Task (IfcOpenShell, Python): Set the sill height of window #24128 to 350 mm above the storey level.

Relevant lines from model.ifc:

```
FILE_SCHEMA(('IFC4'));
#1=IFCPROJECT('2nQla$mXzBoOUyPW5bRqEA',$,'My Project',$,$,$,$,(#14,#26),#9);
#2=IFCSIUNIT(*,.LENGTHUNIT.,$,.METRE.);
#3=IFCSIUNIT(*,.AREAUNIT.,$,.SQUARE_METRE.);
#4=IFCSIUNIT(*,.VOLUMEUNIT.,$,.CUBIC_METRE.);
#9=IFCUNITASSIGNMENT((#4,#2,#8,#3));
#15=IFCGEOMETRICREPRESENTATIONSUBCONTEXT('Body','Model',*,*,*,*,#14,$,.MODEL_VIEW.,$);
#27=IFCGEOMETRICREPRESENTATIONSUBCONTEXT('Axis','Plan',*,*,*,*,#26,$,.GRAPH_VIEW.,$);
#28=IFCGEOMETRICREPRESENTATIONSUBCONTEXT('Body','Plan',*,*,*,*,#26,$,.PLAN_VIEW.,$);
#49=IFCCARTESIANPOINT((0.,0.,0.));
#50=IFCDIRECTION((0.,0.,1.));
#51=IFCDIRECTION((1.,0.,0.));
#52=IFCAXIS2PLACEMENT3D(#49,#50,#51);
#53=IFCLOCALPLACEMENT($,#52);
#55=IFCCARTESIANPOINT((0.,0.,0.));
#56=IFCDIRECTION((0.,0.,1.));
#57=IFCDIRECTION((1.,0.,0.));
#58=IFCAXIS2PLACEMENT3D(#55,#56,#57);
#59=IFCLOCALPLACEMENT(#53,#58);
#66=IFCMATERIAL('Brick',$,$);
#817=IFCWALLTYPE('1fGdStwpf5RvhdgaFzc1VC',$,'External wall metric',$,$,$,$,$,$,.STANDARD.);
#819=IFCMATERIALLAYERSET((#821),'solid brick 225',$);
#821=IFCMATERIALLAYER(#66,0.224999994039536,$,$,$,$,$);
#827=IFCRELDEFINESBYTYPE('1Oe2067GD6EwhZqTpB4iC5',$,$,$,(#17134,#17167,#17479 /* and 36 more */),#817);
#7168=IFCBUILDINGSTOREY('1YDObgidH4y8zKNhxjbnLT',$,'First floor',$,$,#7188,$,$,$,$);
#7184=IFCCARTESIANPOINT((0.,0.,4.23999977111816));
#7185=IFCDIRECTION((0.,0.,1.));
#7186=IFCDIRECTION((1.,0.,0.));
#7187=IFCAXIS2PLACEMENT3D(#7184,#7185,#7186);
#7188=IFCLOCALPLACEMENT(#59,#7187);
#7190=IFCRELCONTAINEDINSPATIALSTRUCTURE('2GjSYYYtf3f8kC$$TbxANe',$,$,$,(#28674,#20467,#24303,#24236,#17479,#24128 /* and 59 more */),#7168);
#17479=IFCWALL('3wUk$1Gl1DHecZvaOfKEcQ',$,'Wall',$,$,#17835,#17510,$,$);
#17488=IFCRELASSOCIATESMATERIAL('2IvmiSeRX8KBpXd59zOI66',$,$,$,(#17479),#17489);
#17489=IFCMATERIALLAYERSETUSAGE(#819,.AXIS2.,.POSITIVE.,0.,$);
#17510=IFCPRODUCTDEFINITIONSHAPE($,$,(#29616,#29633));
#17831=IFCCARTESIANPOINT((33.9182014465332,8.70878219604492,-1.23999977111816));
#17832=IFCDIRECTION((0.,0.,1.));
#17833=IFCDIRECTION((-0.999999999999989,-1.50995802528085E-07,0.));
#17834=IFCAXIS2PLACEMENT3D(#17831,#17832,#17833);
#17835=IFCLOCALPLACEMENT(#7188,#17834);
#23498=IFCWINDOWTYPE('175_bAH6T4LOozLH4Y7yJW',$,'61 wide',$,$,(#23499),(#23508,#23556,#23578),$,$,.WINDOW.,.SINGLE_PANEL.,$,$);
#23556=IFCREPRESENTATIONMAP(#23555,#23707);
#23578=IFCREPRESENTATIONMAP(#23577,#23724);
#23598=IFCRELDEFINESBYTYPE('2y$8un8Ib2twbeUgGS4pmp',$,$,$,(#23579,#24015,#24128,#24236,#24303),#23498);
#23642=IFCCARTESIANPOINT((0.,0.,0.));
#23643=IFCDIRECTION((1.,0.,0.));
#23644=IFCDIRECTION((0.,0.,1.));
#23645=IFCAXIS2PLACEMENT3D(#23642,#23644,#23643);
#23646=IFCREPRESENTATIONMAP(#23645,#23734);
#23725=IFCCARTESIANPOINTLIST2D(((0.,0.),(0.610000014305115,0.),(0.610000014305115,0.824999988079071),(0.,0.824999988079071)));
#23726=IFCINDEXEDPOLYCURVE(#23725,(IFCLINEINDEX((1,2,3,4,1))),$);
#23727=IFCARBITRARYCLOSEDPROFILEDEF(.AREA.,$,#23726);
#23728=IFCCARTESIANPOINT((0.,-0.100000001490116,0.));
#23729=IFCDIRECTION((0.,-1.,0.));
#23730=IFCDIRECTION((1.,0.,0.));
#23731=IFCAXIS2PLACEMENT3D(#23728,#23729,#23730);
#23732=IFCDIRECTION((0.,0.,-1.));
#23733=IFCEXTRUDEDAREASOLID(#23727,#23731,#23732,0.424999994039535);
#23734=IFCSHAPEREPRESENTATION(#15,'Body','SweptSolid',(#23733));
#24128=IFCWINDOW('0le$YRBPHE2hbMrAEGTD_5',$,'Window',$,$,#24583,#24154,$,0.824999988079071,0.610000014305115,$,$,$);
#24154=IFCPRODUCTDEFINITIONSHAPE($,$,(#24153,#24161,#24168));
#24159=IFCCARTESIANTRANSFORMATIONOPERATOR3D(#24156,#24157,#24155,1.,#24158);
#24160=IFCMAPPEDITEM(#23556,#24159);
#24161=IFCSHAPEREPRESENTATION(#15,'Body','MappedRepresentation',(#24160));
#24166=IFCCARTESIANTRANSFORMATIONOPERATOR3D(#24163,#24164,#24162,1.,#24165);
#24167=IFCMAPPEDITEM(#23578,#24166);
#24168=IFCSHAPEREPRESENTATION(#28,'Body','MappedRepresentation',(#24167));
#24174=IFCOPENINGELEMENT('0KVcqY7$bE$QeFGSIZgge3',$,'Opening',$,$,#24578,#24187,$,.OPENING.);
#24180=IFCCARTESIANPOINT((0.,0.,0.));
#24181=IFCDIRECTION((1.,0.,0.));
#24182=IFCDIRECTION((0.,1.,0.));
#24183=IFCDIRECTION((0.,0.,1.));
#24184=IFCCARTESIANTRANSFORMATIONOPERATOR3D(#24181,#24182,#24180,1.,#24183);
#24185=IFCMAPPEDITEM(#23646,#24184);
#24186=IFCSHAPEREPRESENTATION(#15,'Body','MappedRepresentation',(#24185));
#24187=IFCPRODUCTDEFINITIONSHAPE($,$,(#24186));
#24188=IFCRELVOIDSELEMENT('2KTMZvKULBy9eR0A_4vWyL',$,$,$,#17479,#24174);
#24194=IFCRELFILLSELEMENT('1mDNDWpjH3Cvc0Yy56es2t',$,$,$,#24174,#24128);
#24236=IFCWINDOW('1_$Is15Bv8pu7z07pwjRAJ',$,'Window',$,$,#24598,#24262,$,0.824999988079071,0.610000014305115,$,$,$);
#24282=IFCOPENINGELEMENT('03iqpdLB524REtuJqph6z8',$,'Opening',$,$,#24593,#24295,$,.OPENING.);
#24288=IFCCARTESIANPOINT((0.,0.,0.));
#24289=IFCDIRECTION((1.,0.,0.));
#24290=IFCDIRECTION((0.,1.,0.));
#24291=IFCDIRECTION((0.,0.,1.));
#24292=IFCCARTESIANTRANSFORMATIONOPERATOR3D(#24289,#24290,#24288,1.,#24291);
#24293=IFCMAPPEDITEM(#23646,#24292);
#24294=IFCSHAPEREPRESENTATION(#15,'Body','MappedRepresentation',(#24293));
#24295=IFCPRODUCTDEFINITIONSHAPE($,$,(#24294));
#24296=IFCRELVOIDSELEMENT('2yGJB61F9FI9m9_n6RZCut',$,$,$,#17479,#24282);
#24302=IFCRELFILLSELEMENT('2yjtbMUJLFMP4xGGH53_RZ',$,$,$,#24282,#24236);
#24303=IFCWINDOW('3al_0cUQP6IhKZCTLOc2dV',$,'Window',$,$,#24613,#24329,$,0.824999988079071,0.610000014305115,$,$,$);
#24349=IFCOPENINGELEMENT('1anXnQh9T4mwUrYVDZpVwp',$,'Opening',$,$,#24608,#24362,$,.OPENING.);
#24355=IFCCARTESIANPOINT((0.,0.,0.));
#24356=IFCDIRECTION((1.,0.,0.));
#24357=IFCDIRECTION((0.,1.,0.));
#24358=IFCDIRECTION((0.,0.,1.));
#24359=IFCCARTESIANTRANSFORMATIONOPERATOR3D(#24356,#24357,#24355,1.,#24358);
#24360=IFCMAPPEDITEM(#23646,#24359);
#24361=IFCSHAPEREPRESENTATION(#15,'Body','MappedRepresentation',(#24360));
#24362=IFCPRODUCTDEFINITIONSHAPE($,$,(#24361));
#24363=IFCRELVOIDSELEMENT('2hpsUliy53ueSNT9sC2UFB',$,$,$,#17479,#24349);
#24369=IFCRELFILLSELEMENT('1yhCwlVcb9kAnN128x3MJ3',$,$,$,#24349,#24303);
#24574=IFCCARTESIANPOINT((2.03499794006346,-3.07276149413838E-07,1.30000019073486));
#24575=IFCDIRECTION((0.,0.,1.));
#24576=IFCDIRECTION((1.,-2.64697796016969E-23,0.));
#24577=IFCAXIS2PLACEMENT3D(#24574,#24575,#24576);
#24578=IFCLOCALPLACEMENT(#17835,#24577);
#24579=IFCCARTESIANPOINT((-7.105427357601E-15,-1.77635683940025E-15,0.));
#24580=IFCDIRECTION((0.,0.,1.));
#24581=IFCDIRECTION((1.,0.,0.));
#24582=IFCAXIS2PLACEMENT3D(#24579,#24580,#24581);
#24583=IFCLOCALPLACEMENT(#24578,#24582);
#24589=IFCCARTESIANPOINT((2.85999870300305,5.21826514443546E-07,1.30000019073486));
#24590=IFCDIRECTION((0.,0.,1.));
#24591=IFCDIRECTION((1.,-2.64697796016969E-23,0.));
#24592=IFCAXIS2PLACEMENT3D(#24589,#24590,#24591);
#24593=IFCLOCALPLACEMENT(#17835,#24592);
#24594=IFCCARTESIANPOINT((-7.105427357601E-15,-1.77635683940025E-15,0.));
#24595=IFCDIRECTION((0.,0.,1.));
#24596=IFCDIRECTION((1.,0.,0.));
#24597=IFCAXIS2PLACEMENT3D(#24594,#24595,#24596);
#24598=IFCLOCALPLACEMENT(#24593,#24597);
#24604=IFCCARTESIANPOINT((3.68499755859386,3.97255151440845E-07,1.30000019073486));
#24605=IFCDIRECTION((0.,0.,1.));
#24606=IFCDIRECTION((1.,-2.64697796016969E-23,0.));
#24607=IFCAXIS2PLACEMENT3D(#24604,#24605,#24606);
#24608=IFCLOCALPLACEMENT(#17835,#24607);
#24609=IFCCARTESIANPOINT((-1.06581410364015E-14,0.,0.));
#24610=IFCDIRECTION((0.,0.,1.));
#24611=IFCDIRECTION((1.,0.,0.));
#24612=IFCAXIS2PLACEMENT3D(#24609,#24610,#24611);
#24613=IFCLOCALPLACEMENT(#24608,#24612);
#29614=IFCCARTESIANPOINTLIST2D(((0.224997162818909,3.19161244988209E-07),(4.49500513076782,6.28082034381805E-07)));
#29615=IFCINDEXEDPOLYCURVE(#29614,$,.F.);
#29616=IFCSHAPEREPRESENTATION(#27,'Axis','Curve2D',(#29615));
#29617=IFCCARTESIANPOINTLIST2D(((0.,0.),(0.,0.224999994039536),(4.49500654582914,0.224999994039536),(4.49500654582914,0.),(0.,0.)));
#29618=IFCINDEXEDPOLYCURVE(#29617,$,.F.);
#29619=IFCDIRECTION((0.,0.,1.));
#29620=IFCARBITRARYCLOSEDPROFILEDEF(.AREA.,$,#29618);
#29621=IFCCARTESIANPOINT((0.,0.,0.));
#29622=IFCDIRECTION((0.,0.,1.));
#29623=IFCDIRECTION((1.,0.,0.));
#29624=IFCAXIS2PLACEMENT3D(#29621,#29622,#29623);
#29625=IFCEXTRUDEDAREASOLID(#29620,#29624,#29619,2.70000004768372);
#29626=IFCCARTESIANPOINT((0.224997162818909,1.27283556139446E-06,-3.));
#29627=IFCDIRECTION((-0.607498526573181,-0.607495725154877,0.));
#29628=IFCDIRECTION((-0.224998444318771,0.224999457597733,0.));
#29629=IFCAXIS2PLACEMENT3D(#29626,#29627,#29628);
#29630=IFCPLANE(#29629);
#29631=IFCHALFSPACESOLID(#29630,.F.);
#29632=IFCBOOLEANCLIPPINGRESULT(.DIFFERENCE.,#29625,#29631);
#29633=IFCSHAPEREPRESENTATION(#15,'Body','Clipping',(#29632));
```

```python
import numpy as np
import ifcopenshell
import ifcopenshell.api.geometry
import ifcopenshell.geom
import ifcopenshell.util.element
import ifcopenshell.util.placement
import ifcopenshell.util.shape
import ifcopenshell.util.unit

model = ifcopenshell.open("model.ifc")
unit_scale = ifcopenshell.util.unit.calculate_unit_scale(model)

window = model.by_id(24128)
opening = window.FillsVoids[0].RelatingOpeningElement
storey = ifcopenshell.util.element.get_container(window, ifc_class="IfcBuildingStorey")
level = ifcopenshell.util.placement.get_local_placement(storey.ObjectPlacement)[2, 3]

# The opening's origin need not be at the sill, so measure its lowest point.
shape = ifcopenshell.geom.create_shape(ifcopenshell.geom.settings(), opening)
bottom = ifcopenshell.util.shape.get_shape_bottom_elevation(shape, shape.geometry) / unit_scale
dz = level + 0.35 / unit_scale - bottom

shift = np.array([0.0, 0.0, dz])
# The window is placed relative to its opening, so it follows when the opening moves.
matrix = ifcopenshell.util.placement.get_local_placement(opening.ObjectPlacement)
matrix[:3, 3] += shift
ifcopenshell.api.geometry.edit_object_placement(
    model, product=opening, matrix=matrix, is_si=False, should_transform_children=True
)

print(f"moved by {dz * unit_scale:+.3f} m")

model.write("model_edited.ifc")
```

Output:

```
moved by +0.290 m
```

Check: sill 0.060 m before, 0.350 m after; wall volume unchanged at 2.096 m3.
